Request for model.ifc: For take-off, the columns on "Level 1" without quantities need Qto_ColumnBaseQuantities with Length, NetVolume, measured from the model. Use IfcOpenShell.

First a look at what the model holds.

```python
import ifcopenshell
import ifcopenshell.util.element
import ifcopenshell.util.unit

model = ifcopenshell.open("model.ifc")
print(model.schema)
for unit_type in ("LENGTHUNIT", "AREAUNIT", "VOLUMEUNIT"):
    print(unit_type, ifcopenshell.util.unit.calculate_unit_scale(model, unit_type))
storey = next(s for s in model.by_type("IfcBuildingStorey") if s.Name == "Level 1")
columns = [e for e in ifcopenshell.util.element.get_decomposition(storey) if e.is_a("IfcColumn")]
for e in sorted(columns, key=lambda e: e.id()):
    print(e.id(), e.is_a(), e.Name, list(ifcopenshell.util.element.get_psets(e, qtos_only=True)), sep=" | ")
```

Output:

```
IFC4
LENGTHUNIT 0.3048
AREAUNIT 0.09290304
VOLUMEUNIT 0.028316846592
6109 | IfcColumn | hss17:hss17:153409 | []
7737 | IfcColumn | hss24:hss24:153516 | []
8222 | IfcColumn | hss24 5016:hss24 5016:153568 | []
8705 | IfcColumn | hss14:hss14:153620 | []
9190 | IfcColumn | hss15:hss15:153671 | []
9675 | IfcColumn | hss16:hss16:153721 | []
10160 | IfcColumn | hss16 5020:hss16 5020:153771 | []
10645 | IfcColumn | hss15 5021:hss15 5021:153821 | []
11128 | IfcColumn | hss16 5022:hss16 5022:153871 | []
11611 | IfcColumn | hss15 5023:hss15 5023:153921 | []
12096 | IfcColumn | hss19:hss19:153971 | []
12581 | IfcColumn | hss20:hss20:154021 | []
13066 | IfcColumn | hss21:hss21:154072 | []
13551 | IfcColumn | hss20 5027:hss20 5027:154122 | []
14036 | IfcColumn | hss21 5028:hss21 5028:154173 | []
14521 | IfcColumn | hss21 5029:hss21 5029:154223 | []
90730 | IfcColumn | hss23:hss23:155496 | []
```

```python
import ifcopenshell
import ifcopenshell.api.pset
import ifcopenshell.geom
import ifcopenshell.util.element
import ifcopenshell.util.shape
import ifcopenshell.util.unit

model = ifcopenshell.open("model.ifc")
unit_scale = ifcopenshell.util.unit.calculate_unit_scale(model)
volume_scale = ifcopenshell.util.unit.calculate_unit_scale(model, "VOLUMEUNIT")
settings = ifcopenshell.geom.settings()

storey = next(s for s in model.by_type("IfcBuildingStorey") if s.Name == "Level 1")
columns = [e for e in ifcopenshell.util.element.get_decomposition(storey) if e.is_a("IfcColumn")]

for e in sorted(columns, key=lambda e: e.id()):
    if ifcopenshell.util.element.get_psets(e, qtos_only=True, should_inherit=False):
        continue
    # Geometry comes back in metres, in the element's own axes.
    shape = ifcopenshell.geom.create_shape(settings, e)
    values = {
        "Length": ifcopenshell.util.shape.get_z(shape.geometry) / unit_scale,
        "NetVolume": ifcopenshell.util.shape.get_volume(shape.geometry) / volume_scale,
    }
    qto = ifcopenshell.api.pset.add_qto(model, product=e, name="Qto_ColumnBaseQuantities")
    ifcopenshell.api.pset.edit_qto(model, qto=qto, properties=values)
    print(e.id(), {k: round(v, 3) for k, v in values.items()})

model.write("model_rev.ifc")
```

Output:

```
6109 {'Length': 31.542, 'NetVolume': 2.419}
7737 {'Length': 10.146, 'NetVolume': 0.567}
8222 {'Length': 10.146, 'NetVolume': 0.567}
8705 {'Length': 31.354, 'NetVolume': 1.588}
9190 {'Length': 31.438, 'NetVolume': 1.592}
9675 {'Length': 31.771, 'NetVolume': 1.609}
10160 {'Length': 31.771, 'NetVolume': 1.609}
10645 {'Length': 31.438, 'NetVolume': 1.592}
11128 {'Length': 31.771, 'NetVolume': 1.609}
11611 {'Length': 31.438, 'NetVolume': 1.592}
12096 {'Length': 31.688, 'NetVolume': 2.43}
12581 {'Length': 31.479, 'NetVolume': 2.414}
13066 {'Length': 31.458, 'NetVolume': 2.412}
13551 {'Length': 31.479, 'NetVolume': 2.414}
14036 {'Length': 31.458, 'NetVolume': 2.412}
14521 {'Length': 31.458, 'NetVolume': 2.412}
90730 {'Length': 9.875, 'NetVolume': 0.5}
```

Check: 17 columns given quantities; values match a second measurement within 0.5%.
